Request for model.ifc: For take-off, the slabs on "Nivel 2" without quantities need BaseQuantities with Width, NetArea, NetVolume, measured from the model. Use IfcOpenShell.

First a look at what the model holds.

```python
import ifcopenshell
import ifcopenshell.util.element
import ifcopenshell.util.unit

model = ifcopenshell.open("model.ifc")
print(model.schema)
for unit_type in ("LENGTHUNIT", "AREAUNIT", "VOLUMEUNIT"):
    print(unit_type, ifcopenshell.util.unit.calculate_unit_scale(model, unit_type))
storey = next(s for s in model.by_type("IfcBuildingStorey") if s.Name == "Nivel 2")
slabs = [e for e in ifcopenshell.util.element.get_decomposition(storey) if e.is_a("IfcSlab")]
for e in sorted(slabs, key=lambda e: e.id()):
    print(e.id(), e.is_a(), e.Name, list(ifcopenshell.util.element.get_psets(e, qtos_only=True)), sep=" | ")
```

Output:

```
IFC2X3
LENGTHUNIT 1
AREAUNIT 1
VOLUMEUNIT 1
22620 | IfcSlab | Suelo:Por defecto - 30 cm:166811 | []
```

```python
import ifcopenshell
import ifcopenshell.api.pset
import ifcopenshell.geom
import ifcopenshell.util.element
import ifcopenshell.util.shape
import ifcopenshell.util.unit

model = ifcopenshell.open("model.ifc")
unit_scale = ifcopenshell.util.unit.calculate_unit_scale(model)
area_scale = ifcopenshell.util.unit.calculate_unit_scale(model, "AREAUNIT")
volume_scale = ifcopenshell.util.unit.calculate_unit_scale(model, "VOLUMEUNIT")
settings = ifcopenshell.geom.settings()

storey = next(s for s in model.by_type("IfcBuildingStorey") if s.Name == "Nivel 2")
slabs = [e for e in ifcopenshell.util.element.get_decomposition(storey) if e.is_a("IfcSlab")]

for e in sorted(slabs, key=lambda e: e.id()):
    if ifcopenshell.util.element.get_psets(e, qtos_only=True, should_inherit=False):
        continue
    # Geometry comes back in metres, in the element's own axes.
    shape = ifcopenshell.geom.create_shape(settings, e)
    values = {
        "Width": ifcopenshell.util.shape.get_z(shape.geometry) / unit_scale,
        "NetArea": ifcopenshell.util.shape.get_footprint_area(shape.geometry) / area_scale,
        "NetVolume": ifcopenshell.util.shape.get_volume(shape.geometry) / volume_scale,
    }
    qto = ifcopenshell.api.pset.add_qto(model, product=e, name="BaseQuantities")
    ifcopenshell.api.pset.edit_qto(model, qto=qto, properties=values)
    print(e.id(), {k: round(v, 3) for k, v in values.items()})

model.write("model_rev.ifc")
```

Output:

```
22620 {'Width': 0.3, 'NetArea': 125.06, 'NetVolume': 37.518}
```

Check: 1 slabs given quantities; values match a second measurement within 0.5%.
